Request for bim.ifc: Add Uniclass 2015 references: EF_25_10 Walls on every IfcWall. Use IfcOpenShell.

First a look at what the model holds.

```python
import ifcopenshell

model = ifcopenshell.open("bim.ifc")
print(model.schema)
print("classifications:", [c.Name for c in model.by_type("IfcClassification")])
for ifc_class in ("IfcDoor", "IfcRoof", "IfcStair", "IfcWall", "IfcWindow"):
    print(ifc_class, len(model.by_type(ifc_class)))
```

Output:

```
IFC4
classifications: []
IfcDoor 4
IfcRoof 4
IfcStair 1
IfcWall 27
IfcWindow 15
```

```python
import ifcopenshell
import ifcopenshell.api.classification

model = ifcopenshell.open("bim.ifc")

system = ifcopenshell.api.classification.add_classification(model, classification="Uniclass 2015")

codes = {
    "IfcWall": ("EF_25_10", "Walls"),
}
for ifc_class, (code, name) in codes.items():
    products = model.by_type(ifc_class)
    ifcopenshell.api.classification.add_reference(
        model, products=products, classification=system, identification=code, name=name
    )
    print(code, len(products))

model.write("bim_edited.ifc")
```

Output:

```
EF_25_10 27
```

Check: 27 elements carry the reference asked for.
